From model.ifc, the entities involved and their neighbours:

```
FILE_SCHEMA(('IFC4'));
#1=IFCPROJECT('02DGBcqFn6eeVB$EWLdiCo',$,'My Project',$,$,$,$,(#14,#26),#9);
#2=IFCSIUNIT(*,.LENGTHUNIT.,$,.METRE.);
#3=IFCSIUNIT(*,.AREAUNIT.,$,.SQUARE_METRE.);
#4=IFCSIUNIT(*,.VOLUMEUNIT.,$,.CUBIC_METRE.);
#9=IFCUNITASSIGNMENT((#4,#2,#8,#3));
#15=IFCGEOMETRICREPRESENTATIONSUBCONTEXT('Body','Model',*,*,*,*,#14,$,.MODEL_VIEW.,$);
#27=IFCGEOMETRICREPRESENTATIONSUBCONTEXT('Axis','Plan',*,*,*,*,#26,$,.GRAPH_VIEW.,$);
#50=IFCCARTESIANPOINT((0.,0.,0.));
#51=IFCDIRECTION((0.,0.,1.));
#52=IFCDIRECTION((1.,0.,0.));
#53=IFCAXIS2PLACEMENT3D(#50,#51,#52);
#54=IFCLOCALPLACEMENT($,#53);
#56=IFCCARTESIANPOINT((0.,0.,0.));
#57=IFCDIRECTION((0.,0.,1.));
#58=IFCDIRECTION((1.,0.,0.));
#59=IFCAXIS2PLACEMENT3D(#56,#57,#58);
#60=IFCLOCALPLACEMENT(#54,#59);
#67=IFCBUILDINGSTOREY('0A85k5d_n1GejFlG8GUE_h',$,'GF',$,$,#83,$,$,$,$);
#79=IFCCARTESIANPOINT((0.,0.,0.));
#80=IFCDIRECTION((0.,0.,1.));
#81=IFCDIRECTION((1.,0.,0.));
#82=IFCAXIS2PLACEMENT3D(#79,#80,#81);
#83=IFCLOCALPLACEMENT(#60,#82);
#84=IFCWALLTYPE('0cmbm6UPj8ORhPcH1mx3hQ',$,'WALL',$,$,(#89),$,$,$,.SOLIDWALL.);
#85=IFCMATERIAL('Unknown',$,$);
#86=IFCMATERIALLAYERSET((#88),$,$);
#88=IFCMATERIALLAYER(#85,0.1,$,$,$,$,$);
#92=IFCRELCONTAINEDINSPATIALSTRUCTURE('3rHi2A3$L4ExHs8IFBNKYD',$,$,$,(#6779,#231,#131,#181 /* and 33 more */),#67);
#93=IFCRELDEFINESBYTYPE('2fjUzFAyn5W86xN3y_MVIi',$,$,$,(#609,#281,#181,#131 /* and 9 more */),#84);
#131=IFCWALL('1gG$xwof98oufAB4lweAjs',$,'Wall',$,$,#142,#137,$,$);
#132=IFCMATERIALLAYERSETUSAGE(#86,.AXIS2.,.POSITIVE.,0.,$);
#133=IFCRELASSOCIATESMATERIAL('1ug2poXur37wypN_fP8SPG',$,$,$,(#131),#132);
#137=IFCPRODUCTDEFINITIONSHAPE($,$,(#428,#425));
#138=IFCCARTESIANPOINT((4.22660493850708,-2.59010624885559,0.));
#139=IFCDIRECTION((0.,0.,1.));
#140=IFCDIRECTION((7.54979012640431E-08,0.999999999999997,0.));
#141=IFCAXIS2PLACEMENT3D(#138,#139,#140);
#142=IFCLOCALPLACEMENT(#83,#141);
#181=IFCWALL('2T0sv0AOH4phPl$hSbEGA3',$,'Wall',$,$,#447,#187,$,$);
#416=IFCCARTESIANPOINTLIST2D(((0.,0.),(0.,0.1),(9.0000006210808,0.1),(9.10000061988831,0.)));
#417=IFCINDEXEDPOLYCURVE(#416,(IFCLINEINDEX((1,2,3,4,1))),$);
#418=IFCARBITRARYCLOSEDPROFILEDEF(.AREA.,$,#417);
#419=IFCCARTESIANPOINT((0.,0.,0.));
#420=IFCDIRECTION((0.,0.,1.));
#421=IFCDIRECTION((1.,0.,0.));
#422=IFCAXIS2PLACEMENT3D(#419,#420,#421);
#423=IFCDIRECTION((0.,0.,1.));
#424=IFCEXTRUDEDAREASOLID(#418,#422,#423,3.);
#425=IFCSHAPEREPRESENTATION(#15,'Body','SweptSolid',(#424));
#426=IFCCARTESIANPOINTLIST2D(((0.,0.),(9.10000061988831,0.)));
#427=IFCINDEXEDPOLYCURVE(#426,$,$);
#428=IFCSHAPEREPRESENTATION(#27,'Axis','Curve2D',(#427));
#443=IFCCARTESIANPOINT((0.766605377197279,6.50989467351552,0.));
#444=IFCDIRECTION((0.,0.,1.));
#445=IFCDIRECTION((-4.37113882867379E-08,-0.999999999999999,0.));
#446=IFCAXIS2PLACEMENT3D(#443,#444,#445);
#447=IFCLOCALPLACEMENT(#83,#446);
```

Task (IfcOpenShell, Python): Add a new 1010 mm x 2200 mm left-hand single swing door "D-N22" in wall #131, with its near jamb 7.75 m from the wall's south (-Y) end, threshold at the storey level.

```python
import numpy as np
import ifcopenshell
import ifcopenshell.api.feature
import ifcopenshell.api.geometry
import ifcopenshell.api.root
import ifcopenshell.api.spatial
import ifcopenshell.geom
import ifcopenshell.util.element
import ifcopenshell.util.placement
import ifcopenshell.util.representation
import ifcopenshell.util.shape
import ifcopenshell.util.unit

model = ifcopenshell.open("model.ifc")
unit_scale = ifcopenshell.util.unit.calculate_unit_scale(model)
settings = ifcopenshell.geom.settings()


def volume(element):
    """Net volume in cubic metres, openings subtracted."""
    shape = ifcopenshell.geom.create_shape(settings, element)
    return ifcopenshell.util.shape.get_volume(shape.geometry)


wall = model.by_guid("1gG$xwof98oufAB4lweAjs")
storey = ifcopenshell.util.element.get_container(wall, ifc_class="IfcBuildingStorey")
context = ifcopenshell.util.representation.get_context(model, "Model", "Body", "MODEL_VIEW")
before = volume(wall)

width, height, from_end, sill = 1.01, 2.2, 7.75, 0.0  # metres

# The wall runs along its own X axis, and the end named is its -X end.
wall_shape = ifcopenshell.geom.create_shape(settings, wall)
x, y, z = ifcopenshell.util.shape.get_vertices(wall_shape.geometry).T
start = x.min() + from_end
face, thickness = float(y.min()), float(y.max() - y.min())
wall_matrix = ifcopenshell.util.placement.get_local_placement(wall.ObjectPlacement)
level = ifcopenshell.util.placement.get_local_placement(storey.ObjectPlacement)[2, 3]


def in_wall(x, y):
    """Placement at x, y metres in the wall's axes, at sill height."""
    matrix = wall_matrix.copy()
    matrix[:, 3] = wall_matrix @ np.array([x / unit_scale, y / unit_scale, 0.0, 1.0])
    matrix[2, 3] = level + sill / unit_scale
    return matrix


# Opening: a box that overshoots both wall faces by 50 mm.
opening = ifcopenshell.api.root.create_entity(model, ifc_class="IfcOpeningElement", predefined_type="OPENING")
box = ifcopenshell.api.geometry.add_wall_representation(
    model, context=context, length=width, height=height, thickness=thickness + 0.1
)
ifcopenshell.api.geometry.assign_representation(model, product=opening, representation=box)
ifcopenshell.api.geometry.edit_object_placement(model, product=opening, matrix=in_wall(start, face - 0.05), is_si=False)
ifcopenshell.api.feature.add_feature(model, feature=opening, element=wall)

door = ifcopenshell.api.root.create_entity(model, ifc_class="IfcDoor", name="D-N22", predefined_type="DOOR")
door.OverallWidth, door.OverallHeight = width / unit_scale, height / unit_scale
door.OperationType = "SINGLE_SWING_LEFT"
body = ifcopenshell.api.geometry.add_door_representation(
    model,
    context=context,
    overall_width=door.OverallWidth,
    overall_height=door.OverallHeight,
    operation_type="SINGLE_SWING_LEFT",
    lining_properties={"LiningDepth": thickness / unit_scale, "ThresholdDepth": thickness / unit_scale},
)
ifcopenshell.api.geometry.assign_representation(model, product=door, representation=body)
ifcopenshell.api.spatial.assign_container(model, products=[door], relating_structure=storey)
ifcopenshell.api.feature.add_filling(model, opening=opening, element=door)

# The lining spans the wall, so the door starts at the wall face.
ifcopenshell.api.geometry.edit_object_placement(model, product=door, matrix=in_wall(start, face), is_si=False)

after = volume(wall)

print(f"wall volume {before:.3f} -> {after:.3f} m3")

model.write("model_edited.ifc")
```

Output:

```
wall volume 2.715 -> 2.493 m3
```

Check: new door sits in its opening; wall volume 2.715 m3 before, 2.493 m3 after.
